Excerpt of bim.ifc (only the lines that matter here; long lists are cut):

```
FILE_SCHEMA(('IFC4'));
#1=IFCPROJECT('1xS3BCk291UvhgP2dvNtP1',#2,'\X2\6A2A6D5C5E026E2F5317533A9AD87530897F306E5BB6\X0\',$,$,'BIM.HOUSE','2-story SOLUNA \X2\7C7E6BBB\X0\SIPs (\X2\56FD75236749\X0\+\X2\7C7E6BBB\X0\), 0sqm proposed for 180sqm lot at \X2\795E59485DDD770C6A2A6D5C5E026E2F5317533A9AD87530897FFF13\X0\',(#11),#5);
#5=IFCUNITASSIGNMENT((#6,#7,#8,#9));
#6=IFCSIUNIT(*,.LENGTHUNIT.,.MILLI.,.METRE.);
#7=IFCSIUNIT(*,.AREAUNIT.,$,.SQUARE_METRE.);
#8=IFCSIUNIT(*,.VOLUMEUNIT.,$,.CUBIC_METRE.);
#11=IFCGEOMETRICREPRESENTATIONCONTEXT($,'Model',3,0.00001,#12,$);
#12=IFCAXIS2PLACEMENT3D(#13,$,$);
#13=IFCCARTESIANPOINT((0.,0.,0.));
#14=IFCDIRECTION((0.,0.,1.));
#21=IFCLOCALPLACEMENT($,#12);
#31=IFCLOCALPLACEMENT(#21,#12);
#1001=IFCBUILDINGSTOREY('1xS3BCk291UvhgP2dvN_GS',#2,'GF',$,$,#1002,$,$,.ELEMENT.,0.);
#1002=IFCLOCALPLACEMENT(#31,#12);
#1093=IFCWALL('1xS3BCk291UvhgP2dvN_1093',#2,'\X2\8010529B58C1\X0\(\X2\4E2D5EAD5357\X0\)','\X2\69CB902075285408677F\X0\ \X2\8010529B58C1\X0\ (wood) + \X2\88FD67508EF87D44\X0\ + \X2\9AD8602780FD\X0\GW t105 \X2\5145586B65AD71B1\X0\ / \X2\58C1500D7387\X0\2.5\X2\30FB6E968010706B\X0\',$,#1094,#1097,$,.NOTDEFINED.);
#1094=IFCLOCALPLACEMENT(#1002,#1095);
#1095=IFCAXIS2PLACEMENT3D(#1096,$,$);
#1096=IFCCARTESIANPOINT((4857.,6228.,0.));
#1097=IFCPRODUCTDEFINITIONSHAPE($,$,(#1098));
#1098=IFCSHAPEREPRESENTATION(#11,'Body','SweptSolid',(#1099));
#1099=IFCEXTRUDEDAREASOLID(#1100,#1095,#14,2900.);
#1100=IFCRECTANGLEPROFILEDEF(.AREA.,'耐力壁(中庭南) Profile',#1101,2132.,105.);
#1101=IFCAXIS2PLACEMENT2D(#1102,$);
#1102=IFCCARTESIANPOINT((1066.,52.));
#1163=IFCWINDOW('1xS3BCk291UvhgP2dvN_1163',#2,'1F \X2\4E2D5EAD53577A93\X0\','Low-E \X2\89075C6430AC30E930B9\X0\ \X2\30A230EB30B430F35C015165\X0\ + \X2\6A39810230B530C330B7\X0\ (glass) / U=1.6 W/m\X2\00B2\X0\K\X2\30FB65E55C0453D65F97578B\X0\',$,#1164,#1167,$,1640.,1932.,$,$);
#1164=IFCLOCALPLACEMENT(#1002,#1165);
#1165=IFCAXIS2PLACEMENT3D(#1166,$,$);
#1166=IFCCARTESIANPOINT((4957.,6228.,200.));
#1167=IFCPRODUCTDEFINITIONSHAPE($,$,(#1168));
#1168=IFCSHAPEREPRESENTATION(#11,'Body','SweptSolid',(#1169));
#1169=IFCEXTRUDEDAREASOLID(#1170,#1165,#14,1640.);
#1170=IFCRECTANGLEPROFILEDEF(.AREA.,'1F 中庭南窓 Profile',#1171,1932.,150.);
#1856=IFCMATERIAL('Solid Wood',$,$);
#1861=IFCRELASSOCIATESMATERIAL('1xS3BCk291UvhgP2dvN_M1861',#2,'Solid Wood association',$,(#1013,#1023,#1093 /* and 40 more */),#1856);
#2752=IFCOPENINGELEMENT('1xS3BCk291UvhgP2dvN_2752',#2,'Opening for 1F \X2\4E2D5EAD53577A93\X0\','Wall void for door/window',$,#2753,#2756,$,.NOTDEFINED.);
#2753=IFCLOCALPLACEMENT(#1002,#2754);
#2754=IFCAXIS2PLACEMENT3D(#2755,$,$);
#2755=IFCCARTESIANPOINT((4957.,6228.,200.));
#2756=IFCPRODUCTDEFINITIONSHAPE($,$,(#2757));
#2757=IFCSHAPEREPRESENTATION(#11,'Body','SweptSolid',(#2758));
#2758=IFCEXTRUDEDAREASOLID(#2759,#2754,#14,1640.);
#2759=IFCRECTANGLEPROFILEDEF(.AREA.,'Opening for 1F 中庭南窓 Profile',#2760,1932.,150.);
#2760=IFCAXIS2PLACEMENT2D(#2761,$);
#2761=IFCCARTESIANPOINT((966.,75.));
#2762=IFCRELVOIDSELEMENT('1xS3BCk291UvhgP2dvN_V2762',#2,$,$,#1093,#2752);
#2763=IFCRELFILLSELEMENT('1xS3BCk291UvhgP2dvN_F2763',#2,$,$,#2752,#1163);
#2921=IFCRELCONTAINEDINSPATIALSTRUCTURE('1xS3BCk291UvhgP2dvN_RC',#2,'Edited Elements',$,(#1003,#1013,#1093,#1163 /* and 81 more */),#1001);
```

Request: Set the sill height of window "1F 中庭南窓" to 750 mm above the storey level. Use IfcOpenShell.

```python
import numpy as np
import ifcopenshell
import ifcopenshell.api.geometry
import ifcopenshell.geom
import ifcopenshell.util.element
import ifcopenshell.util.placement
import ifcopenshell.util.shape
import ifcopenshell.util.unit

model = ifcopenshell.open("bim.ifc")
unit_scale = ifcopenshell.util.unit.calculate_unit_scale(model)

window = model.by_id(1163)
opening = window.FillsVoids[0].RelatingOpeningElement
storey = ifcopenshell.util.element.get_container(window, ifc_class="IfcBuildingStorey")
level = ifcopenshell.util.placement.get_local_placement(storey.ObjectPlacement)[2, 3]

# The opening's origin need not be at the sill, so measure its lowest point.
shape = ifcopenshell.geom.create_shape(ifcopenshell.geom.settings(), opening)
bottom = ifcopenshell.util.shape.get_shape_bottom_elevation(shape, shape.geometry) / unit_scale
dz = level + 0.75 / unit_scale - bottom

shift = np.array([0.0, 0.0, dz])
# The window is not placed relative to its opening, so move both.
for product in (opening, window):
    matrix = ifcopenshell.util.placement.get_local_placement(product.ObjectPlacement)
    matrix[:3, 3] += shift
    ifcopenshell.api.geometry.edit_object_placement(model, product=product, matrix=matrix, is_si=False)

print(f"moved by {dz * unit_scale:+.3f} m")

model.write("bim_rev.ifc")
```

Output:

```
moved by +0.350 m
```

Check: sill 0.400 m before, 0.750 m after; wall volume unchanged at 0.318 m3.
